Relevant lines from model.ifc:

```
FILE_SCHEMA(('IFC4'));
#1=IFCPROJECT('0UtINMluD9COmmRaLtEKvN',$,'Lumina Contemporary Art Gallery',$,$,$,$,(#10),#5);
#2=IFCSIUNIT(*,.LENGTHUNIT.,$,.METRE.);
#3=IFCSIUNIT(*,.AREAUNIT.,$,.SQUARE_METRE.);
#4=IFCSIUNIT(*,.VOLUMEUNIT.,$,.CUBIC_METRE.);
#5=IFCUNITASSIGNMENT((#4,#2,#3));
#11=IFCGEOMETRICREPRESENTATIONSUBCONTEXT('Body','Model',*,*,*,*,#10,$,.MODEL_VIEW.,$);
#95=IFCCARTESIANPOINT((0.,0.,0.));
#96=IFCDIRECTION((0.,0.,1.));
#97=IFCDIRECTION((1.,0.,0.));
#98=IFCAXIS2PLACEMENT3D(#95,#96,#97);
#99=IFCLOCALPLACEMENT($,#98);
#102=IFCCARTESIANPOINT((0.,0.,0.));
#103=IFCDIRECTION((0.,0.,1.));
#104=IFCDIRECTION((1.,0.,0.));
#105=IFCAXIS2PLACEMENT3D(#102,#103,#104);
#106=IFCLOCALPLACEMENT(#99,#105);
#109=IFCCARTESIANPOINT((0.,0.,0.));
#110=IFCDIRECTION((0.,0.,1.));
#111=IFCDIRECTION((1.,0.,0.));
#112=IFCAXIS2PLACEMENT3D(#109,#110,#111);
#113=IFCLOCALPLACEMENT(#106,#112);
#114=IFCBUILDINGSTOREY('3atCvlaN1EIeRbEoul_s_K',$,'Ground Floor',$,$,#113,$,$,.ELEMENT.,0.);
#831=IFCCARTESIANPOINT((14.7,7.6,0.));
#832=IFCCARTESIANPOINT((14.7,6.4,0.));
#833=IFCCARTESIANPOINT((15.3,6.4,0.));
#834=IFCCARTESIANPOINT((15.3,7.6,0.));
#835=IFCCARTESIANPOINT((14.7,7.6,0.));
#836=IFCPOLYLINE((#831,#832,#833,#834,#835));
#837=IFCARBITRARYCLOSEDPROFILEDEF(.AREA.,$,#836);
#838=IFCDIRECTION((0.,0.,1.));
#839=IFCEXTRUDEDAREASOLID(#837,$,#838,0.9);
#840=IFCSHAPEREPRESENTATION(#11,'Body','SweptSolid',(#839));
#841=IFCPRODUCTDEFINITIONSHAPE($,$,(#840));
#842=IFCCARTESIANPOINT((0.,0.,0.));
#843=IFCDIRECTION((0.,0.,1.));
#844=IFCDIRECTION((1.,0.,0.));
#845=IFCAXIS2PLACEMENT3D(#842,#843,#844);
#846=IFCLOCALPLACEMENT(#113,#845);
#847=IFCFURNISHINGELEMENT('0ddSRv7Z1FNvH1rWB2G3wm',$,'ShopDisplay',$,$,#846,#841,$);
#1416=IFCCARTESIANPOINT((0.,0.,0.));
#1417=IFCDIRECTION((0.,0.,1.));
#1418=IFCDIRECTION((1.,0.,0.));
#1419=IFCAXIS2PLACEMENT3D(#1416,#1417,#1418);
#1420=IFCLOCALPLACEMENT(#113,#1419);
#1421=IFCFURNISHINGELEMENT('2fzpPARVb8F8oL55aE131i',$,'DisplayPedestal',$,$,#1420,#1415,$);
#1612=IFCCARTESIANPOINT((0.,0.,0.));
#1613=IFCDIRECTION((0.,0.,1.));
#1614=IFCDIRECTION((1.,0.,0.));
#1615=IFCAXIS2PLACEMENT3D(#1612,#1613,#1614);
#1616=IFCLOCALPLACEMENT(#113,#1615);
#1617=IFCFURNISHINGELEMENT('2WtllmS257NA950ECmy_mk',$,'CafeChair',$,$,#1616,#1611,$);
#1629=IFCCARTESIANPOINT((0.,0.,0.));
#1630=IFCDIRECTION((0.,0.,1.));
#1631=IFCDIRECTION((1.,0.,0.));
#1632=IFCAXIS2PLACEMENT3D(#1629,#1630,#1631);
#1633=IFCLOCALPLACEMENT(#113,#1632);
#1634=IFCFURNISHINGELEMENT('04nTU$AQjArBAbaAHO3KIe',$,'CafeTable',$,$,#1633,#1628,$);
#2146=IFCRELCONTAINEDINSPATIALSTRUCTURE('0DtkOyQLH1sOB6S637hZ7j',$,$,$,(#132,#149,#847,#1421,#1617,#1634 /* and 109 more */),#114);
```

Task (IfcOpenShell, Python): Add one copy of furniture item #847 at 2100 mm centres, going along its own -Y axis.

```python
import ifcopenshell
import ifcopenshell.api.geometry
import ifcopenshell.api.root
import ifcopenshell.util.element
import ifcopenshell.util.placement
import ifcopenshell.util.unit

model = ifcopenshell.open("model.ifc")
unit_scale = ifcopenshell.util.unit.calculate_unit_scale(model)

source = model.by_guid("0ddSRv7Z1FNvH1rWB2G3wm")
base = ifcopenshell.util.placement.get_local_placement(source.ObjectPlacement)
step = -base[:3, 1] * 2.1 / unit_scale

for i in range(1, 2):
    copy = ifcopenshell.api.root.copy_class(model, product=source)
    copy.Representation = ifcopenshell.util.element.copy_deep(
        model, source.Representation, exclude=["IfcGeometricRepresentationContext", "IfcRepresentationMap"]
    )
    matrix = base.copy()
    matrix[:3, 3] += i * step
    print("added at", matrix[:3, 3].round(3) + 0.0)
    ifcopenshell.api.geometry.edit_object_placement(model, product=copy, matrix=matrix, is_si=False)

model.write("model_v2.ifc")
```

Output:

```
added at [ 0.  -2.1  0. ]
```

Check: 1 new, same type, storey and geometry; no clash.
